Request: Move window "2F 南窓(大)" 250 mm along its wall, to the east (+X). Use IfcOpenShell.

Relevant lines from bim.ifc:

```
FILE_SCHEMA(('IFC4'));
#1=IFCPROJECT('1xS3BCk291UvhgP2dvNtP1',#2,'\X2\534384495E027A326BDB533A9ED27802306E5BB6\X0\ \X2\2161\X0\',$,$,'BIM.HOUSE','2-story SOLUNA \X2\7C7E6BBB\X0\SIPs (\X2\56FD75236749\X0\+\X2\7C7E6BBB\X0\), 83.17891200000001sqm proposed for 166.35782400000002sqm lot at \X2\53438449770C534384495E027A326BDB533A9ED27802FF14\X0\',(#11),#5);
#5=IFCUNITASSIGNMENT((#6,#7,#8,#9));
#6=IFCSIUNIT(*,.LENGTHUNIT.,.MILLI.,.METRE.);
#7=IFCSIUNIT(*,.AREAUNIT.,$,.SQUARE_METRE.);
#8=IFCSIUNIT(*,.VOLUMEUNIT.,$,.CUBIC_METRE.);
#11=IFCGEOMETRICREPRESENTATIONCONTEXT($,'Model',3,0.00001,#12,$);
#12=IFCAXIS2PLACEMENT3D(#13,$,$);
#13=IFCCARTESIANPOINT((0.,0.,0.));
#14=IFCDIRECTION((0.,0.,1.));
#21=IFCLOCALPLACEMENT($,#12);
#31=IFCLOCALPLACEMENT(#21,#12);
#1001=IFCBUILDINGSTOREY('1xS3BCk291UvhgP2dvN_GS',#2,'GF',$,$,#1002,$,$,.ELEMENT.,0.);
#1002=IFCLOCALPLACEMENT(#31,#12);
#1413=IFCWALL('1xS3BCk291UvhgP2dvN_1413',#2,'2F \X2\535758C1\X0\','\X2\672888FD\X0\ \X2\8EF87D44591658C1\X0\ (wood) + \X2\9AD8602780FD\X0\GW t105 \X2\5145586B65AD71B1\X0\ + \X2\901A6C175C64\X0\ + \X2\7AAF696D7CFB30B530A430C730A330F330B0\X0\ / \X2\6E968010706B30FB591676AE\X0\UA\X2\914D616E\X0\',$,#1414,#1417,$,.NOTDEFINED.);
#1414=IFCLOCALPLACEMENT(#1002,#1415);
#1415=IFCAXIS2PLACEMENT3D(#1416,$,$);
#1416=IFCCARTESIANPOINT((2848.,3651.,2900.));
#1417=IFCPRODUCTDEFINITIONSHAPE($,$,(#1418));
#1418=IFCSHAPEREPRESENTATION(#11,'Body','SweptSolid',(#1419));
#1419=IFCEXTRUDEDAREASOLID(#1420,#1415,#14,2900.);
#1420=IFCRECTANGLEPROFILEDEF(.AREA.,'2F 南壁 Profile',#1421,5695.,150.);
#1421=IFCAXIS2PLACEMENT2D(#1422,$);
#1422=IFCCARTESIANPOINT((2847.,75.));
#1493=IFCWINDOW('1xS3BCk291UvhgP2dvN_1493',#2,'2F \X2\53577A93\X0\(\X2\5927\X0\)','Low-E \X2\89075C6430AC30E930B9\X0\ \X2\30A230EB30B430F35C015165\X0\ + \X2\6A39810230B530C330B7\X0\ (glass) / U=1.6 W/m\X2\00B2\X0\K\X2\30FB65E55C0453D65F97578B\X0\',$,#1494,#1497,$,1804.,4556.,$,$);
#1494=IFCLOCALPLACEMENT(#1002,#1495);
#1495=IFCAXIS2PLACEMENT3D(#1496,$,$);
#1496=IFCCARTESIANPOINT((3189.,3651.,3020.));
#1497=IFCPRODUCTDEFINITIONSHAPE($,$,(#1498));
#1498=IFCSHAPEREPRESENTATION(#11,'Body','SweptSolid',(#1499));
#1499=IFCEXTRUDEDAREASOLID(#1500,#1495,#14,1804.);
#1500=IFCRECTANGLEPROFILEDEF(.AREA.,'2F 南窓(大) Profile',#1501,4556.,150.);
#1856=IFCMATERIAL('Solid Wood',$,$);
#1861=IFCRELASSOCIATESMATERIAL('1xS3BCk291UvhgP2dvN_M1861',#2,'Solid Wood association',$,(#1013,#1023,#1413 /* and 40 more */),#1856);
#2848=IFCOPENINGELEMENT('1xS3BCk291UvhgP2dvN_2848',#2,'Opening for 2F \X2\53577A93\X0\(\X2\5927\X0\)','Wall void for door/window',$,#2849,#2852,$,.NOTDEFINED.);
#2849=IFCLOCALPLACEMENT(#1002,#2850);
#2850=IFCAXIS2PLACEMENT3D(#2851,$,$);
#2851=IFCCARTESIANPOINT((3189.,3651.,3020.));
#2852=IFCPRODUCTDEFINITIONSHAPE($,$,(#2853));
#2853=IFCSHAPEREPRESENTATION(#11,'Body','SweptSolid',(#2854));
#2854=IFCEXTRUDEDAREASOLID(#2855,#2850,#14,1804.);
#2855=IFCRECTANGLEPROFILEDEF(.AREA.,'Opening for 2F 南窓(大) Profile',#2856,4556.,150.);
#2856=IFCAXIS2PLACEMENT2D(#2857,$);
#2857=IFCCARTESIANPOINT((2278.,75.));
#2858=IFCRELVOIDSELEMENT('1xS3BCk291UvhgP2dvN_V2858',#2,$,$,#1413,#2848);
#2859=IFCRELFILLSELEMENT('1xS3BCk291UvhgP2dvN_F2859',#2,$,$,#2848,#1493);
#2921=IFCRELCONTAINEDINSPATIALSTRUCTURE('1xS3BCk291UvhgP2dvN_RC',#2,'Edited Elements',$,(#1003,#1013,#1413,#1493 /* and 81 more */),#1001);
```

```python
import ifcopenshell
import ifcopenshell.api.geometry
import ifcopenshell.util.placement

model = ifcopenshell.open("bim.ifc")

window = model.by_id(1493)
opening = window.FillsVoids[0].RelatingOpeningElement
wall = opening.VoidsElements[0].RelatingBuildingElement

wall_matrix = ifcopenshell.util.placement.get_local_placement(wall.ObjectPlacement)
shift = wall_matrix[:3, 0] * 250.0
before = ifcopenshell.util.placement.get_local_placement(window.ObjectPlacement)[:3, 3].copy()

# The window is not placed relative to its opening, so move both.
for product in (opening, window):
    matrix = ifcopenshell.util.placement.get_local_placement(product.ObjectPlacement)
    matrix[:3, 3] += shift
    ifcopenshell.api.geometry.edit_object_placement(model, product=product, matrix=matrix, is_si=False)

after = ifcopenshell.util.placement.get_local_placement(window.ObjectPlacement)[:3, 3]
print("window moved by", (after - before).round(3) + 0.0)

model.write("bim_updated.ifc")
```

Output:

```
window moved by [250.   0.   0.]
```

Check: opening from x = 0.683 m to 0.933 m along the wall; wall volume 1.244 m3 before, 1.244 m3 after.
